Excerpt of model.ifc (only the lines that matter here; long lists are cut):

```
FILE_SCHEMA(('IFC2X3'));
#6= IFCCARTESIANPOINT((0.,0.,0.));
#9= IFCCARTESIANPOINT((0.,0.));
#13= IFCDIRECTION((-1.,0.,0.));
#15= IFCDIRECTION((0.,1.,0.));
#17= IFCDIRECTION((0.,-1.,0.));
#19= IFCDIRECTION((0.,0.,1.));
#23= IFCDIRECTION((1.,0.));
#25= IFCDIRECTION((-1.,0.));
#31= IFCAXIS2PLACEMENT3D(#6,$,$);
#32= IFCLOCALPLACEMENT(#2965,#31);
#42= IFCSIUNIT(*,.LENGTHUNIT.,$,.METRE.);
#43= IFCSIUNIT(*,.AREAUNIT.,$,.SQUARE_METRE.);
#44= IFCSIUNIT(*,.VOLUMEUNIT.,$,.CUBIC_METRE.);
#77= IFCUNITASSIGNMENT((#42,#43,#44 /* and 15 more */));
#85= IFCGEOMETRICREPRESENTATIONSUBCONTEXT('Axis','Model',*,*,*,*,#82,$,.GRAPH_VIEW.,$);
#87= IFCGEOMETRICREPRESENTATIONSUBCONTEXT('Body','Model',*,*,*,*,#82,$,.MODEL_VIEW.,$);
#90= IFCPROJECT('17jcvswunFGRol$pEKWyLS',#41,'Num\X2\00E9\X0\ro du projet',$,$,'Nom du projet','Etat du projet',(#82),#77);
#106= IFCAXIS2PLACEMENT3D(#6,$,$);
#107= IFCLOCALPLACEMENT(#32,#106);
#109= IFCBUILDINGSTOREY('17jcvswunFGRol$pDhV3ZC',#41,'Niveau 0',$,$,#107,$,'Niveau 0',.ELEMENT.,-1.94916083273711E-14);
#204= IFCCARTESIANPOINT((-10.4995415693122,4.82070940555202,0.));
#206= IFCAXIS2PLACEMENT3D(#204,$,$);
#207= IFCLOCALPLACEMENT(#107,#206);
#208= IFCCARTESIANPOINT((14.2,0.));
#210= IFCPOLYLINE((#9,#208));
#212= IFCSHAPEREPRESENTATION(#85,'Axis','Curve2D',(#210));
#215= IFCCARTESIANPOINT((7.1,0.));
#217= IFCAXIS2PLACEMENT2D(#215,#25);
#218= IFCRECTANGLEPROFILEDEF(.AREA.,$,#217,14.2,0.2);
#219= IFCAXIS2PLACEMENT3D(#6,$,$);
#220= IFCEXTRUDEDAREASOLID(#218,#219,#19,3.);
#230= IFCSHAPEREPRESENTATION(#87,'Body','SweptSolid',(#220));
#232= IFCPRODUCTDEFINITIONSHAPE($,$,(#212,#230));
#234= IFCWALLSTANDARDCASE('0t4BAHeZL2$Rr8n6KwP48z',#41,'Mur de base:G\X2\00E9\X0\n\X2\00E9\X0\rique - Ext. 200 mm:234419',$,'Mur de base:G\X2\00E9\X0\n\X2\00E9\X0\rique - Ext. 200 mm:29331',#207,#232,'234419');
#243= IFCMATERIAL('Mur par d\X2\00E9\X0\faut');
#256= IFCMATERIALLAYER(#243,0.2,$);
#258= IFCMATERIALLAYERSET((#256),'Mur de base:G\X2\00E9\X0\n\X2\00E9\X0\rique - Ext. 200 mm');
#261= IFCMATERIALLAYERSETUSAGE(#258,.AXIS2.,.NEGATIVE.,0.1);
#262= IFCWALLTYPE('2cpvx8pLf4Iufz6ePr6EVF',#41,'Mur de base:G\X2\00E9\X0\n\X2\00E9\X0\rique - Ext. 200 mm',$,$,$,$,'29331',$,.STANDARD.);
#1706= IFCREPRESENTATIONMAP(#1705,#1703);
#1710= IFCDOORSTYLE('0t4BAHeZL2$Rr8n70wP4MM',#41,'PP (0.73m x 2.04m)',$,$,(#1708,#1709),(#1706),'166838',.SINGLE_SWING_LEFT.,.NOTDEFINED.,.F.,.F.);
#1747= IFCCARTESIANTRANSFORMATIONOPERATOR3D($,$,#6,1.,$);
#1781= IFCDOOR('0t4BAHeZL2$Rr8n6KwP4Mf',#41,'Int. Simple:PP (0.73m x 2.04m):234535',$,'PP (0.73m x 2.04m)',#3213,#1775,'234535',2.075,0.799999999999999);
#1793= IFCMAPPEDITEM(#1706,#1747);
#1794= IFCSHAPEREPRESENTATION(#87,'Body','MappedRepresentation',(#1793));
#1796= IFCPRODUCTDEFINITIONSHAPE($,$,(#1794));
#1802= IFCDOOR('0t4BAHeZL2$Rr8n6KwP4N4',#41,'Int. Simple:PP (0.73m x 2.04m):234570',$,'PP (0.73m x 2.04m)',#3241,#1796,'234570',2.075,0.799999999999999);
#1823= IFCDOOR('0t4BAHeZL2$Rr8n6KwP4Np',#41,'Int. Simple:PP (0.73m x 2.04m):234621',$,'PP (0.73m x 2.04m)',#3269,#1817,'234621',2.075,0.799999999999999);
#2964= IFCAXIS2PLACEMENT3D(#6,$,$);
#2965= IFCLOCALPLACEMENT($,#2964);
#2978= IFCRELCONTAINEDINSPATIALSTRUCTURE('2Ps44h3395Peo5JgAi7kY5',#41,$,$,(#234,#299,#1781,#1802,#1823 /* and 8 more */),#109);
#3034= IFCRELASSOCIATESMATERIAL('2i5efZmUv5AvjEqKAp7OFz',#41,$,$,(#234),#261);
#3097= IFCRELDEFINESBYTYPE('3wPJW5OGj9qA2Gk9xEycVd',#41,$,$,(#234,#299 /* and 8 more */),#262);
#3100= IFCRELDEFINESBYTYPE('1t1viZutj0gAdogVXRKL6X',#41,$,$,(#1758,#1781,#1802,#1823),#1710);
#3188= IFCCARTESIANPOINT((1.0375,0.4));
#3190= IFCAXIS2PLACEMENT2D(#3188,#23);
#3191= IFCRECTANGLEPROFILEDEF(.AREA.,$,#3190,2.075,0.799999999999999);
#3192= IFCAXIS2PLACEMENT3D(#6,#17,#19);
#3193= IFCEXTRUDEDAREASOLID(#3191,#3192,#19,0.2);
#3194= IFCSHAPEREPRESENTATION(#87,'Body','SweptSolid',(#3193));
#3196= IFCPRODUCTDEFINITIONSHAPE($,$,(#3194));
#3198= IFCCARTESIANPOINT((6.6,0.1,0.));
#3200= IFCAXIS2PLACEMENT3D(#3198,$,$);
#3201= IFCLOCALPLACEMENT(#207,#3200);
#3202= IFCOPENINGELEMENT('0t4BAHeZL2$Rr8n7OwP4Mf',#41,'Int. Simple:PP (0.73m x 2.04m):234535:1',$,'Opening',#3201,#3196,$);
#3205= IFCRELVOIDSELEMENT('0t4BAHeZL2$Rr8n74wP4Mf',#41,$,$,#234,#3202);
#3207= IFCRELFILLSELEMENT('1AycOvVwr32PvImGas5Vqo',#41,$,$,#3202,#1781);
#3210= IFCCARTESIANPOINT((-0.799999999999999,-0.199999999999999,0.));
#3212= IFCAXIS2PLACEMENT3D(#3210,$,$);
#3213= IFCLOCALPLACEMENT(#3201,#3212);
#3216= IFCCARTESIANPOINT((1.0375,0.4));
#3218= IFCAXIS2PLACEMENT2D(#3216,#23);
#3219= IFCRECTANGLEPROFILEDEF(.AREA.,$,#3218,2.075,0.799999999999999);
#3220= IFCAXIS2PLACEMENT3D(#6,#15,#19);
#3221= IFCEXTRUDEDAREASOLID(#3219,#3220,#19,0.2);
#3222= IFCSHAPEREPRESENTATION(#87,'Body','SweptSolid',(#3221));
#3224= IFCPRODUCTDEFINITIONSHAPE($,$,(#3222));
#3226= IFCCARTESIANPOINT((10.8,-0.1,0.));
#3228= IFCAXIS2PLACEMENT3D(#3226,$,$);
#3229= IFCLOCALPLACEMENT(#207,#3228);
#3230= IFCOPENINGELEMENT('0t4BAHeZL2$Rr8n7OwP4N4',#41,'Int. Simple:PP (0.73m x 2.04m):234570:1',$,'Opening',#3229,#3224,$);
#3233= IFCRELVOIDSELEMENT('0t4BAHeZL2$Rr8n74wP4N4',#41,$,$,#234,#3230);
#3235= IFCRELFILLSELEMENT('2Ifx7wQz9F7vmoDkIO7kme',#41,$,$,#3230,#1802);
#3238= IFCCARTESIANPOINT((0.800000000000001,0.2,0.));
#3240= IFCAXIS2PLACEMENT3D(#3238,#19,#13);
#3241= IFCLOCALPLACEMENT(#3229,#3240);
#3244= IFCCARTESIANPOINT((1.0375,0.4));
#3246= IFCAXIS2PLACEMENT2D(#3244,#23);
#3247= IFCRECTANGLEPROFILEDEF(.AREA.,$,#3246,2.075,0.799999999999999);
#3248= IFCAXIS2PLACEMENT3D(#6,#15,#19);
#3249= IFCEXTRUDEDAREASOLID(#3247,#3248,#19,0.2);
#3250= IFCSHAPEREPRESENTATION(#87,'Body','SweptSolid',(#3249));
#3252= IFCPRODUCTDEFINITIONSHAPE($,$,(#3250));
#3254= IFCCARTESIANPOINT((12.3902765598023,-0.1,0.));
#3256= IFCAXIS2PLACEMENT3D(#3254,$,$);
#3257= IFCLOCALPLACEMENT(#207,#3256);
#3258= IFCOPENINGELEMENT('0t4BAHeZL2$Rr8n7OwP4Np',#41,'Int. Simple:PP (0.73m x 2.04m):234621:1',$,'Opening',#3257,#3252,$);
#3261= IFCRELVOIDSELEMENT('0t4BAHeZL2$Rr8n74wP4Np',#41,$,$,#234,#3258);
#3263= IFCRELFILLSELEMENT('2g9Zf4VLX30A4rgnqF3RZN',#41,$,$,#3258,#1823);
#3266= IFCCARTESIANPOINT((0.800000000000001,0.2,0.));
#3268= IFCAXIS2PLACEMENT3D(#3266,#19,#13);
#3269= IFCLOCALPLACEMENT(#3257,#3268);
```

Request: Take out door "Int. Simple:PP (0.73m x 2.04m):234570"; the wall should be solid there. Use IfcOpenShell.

```python
import ifcopenshell
import ifcopenshell.api.feature
import ifcopenshell.api.root
import ifcopenshell.geom
import ifcopenshell.util.shape

model = ifcopenshell.open("model.ifc")
settings = ifcopenshell.geom.settings()


def volume(element):
    """Net volume in cubic metres, openings subtracted."""
    shape = ifcopenshell.geom.create_shape(settings, element)
    return ifcopenshell.util.shape.get_volume(shape.geometry)


door = model.by_guid("0t4BAHeZL2$Rr8n6KwP4N4")
opening = door.FillsVoids[0].RelatingOpeningElement
wall = opening.VoidsElements[0].RelatingBuildingElement
before = volume(wall)

ifcopenshell.api.root.remove_product(model, product=door)
ifcopenshell.api.feature.remove_feature(model, feature=opening)

after = volume(wall)

print(f"wall volume {before:.3f} -> {after:.3f} m3")

model.write("model_v2.ifc")
```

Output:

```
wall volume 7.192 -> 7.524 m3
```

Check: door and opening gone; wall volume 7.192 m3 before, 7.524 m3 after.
